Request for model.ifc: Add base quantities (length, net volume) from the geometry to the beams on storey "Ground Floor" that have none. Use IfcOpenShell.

First a look at what the model holds.

```python
import ifcopenshell
import ifcopenshell.util.element
import ifcopenshell.util.unit

model = ifcopenshell.open("model.ifc")
print(model.schema)
for unit_type in ("LENGTHUNIT", "AREAUNIT", "VOLUMEUNIT"):
    print(unit_type, ifcopenshell.util.unit.calculate_unit_scale(model, unit_type))
storey = next(s for s in model.by_type("IfcBuildingStorey") if s.Name == "Ground Floor")
beams = [e for e in ifcopenshell.util.element.get_decomposition(storey) if e.is_a("IfcBeam")]
for e in sorted(beams, key=lambda e: e.id()):
    print(e.id(), e.is_a(), e.Name, list(ifcopenshell.util.element.get_psets(e, qtos_only=True)), sep=" | ")
```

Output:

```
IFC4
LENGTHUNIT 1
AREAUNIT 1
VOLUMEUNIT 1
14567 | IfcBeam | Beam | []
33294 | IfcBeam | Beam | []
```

```python
import ifcopenshell
import ifcopenshell.api.pset
import ifcopenshell.geom
import ifcopenshell.util.element
import ifcopenshell.util.shape
import ifcopenshell.util.unit

model = ifcopenshell.open("model.ifc")
unit_scale = ifcopenshell.util.unit.calculate_unit_scale(model)
volume_scale = ifcopenshell.util.unit.calculate_unit_scale(model, "VOLUMEUNIT")
settings = ifcopenshell.geom.settings()

storey = next(s for s in model.by_type("IfcBuildingStorey") if s.Name == "Ground Floor")
beams = [e for e in ifcopenshell.util.element.get_decomposition(storey) if e.is_a("IfcBeam")]

for e in sorted(beams, key=lambda e: e.id()):
    if ifcopenshell.util.element.get_psets(e, qtos_only=True, should_inherit=False):
        continue
    # Geometry comes back in metres, in the element's own axes.
    shape = ifcopenshell.geom.create_shape(settings, e)
    values = {
        "Length": ifcopenshell.util.shape.get_max_xyz(shape.geometry) / unit_scale,
        "NetVolume": ifcopenshell.util.shape.get_volume(shape.geometry) / volume_scale,
    }
    qto = ifcopenshell.api.pset.add_qto(model, product=e, name="Qto_BeamBaseQuantities")
    ifcopenshell.api.pset.edit_qto(model, qto=qto, properties=values)
    print(e.id(), {k: round(v, 3) for k, v in values.items()})

model.write("model_v2.ifc")
```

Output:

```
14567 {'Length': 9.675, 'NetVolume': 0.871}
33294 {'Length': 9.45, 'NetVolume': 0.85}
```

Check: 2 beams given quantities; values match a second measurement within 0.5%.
